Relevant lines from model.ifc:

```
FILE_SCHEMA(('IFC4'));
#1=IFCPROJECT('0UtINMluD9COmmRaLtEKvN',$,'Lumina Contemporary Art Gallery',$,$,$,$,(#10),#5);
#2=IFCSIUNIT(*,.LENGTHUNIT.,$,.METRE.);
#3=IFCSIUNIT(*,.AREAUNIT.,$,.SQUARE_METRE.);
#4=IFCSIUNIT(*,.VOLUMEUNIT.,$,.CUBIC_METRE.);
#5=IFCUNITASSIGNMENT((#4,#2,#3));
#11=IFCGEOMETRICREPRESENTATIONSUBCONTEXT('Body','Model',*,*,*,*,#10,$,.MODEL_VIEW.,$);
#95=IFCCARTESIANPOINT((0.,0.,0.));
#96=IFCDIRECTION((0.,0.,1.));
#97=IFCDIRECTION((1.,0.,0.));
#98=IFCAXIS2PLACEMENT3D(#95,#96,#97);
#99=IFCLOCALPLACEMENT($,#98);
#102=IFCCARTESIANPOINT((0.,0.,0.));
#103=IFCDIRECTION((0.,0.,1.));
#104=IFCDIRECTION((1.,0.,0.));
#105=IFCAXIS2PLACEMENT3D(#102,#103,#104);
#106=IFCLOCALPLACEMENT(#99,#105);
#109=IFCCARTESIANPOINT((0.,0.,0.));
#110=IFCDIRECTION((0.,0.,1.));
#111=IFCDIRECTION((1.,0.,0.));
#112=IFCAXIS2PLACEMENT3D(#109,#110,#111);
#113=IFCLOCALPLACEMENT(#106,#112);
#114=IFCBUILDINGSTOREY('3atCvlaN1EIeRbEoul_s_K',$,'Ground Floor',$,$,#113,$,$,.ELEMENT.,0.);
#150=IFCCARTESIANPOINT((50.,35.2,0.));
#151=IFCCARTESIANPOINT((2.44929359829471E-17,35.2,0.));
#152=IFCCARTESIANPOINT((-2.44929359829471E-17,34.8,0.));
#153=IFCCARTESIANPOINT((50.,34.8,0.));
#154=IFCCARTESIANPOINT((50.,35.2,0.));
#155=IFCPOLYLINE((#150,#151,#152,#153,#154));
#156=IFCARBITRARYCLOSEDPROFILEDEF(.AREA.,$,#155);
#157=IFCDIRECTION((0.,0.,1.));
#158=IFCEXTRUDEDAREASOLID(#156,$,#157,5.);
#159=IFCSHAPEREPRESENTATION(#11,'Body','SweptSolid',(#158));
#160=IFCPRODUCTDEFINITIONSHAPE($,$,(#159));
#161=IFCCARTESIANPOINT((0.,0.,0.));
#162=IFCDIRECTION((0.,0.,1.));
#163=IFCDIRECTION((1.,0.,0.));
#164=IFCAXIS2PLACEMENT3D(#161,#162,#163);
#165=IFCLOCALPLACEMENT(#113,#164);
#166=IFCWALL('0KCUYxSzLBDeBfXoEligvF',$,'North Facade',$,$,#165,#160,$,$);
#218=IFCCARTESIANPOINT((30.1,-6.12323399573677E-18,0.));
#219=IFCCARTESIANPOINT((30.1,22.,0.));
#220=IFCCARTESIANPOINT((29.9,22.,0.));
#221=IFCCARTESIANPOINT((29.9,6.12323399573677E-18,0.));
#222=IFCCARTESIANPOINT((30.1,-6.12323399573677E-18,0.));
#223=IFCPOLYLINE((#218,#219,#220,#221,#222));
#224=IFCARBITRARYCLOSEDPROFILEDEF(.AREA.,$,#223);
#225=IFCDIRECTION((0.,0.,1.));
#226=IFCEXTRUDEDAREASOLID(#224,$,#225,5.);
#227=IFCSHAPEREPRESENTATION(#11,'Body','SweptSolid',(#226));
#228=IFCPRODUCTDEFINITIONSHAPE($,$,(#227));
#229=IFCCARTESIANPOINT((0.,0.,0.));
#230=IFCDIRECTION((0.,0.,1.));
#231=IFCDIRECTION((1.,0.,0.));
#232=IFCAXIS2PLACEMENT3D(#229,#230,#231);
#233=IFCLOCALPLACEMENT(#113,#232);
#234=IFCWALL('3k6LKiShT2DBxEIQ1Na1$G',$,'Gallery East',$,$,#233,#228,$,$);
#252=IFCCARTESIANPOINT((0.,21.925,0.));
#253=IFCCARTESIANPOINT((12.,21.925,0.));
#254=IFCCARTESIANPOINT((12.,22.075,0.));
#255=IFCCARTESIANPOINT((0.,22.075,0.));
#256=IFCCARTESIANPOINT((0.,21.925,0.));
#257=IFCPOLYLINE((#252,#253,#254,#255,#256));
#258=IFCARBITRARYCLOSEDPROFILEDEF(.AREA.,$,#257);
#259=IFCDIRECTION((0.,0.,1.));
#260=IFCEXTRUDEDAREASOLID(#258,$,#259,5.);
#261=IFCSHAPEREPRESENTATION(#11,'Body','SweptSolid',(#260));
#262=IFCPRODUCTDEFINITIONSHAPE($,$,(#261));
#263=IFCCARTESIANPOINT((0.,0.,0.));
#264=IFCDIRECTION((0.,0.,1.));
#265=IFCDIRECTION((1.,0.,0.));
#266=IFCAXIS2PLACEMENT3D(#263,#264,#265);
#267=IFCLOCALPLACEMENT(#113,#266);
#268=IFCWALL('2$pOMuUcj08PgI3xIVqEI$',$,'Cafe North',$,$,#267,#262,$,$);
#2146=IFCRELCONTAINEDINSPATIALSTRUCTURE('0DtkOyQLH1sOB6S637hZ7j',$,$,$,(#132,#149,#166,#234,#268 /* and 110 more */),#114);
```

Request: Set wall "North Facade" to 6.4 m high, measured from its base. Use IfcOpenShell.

```python
import ifcopenshell
import ifcopenshell.geom
import ifcopenshell.util.representation
import ifcopenshell.util.shape

model = ifcopenshell.open("model.ifc")
settings = ifcopenshell.geom.settings()


def volume(element):
    """Net volume in cubic metres, openings subtracted."""
    shape = ifcopenshell.geom.create_shape(settings, element)
    return ifcopenshell.util.shape.get_volume(shape.geometry)


wall = model.by_guid("0KCUYxSzLBDeBfXoEligvF")
before = volume(wall)

body = ifcopenshell.util.representation.get_representation(wall, "Model", "Body")
solid = body.Items[0]
old_height = solid.Depth
solid.Depth = 6.4
after = volume(wall)

print(f"height {old_height:g} -> {solid.Depth:g}, volume {before:.3f} -> {after:.3f} m3")

model.write("model_rev.ifc")
```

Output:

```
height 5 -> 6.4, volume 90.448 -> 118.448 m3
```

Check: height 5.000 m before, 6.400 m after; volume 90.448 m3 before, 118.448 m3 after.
